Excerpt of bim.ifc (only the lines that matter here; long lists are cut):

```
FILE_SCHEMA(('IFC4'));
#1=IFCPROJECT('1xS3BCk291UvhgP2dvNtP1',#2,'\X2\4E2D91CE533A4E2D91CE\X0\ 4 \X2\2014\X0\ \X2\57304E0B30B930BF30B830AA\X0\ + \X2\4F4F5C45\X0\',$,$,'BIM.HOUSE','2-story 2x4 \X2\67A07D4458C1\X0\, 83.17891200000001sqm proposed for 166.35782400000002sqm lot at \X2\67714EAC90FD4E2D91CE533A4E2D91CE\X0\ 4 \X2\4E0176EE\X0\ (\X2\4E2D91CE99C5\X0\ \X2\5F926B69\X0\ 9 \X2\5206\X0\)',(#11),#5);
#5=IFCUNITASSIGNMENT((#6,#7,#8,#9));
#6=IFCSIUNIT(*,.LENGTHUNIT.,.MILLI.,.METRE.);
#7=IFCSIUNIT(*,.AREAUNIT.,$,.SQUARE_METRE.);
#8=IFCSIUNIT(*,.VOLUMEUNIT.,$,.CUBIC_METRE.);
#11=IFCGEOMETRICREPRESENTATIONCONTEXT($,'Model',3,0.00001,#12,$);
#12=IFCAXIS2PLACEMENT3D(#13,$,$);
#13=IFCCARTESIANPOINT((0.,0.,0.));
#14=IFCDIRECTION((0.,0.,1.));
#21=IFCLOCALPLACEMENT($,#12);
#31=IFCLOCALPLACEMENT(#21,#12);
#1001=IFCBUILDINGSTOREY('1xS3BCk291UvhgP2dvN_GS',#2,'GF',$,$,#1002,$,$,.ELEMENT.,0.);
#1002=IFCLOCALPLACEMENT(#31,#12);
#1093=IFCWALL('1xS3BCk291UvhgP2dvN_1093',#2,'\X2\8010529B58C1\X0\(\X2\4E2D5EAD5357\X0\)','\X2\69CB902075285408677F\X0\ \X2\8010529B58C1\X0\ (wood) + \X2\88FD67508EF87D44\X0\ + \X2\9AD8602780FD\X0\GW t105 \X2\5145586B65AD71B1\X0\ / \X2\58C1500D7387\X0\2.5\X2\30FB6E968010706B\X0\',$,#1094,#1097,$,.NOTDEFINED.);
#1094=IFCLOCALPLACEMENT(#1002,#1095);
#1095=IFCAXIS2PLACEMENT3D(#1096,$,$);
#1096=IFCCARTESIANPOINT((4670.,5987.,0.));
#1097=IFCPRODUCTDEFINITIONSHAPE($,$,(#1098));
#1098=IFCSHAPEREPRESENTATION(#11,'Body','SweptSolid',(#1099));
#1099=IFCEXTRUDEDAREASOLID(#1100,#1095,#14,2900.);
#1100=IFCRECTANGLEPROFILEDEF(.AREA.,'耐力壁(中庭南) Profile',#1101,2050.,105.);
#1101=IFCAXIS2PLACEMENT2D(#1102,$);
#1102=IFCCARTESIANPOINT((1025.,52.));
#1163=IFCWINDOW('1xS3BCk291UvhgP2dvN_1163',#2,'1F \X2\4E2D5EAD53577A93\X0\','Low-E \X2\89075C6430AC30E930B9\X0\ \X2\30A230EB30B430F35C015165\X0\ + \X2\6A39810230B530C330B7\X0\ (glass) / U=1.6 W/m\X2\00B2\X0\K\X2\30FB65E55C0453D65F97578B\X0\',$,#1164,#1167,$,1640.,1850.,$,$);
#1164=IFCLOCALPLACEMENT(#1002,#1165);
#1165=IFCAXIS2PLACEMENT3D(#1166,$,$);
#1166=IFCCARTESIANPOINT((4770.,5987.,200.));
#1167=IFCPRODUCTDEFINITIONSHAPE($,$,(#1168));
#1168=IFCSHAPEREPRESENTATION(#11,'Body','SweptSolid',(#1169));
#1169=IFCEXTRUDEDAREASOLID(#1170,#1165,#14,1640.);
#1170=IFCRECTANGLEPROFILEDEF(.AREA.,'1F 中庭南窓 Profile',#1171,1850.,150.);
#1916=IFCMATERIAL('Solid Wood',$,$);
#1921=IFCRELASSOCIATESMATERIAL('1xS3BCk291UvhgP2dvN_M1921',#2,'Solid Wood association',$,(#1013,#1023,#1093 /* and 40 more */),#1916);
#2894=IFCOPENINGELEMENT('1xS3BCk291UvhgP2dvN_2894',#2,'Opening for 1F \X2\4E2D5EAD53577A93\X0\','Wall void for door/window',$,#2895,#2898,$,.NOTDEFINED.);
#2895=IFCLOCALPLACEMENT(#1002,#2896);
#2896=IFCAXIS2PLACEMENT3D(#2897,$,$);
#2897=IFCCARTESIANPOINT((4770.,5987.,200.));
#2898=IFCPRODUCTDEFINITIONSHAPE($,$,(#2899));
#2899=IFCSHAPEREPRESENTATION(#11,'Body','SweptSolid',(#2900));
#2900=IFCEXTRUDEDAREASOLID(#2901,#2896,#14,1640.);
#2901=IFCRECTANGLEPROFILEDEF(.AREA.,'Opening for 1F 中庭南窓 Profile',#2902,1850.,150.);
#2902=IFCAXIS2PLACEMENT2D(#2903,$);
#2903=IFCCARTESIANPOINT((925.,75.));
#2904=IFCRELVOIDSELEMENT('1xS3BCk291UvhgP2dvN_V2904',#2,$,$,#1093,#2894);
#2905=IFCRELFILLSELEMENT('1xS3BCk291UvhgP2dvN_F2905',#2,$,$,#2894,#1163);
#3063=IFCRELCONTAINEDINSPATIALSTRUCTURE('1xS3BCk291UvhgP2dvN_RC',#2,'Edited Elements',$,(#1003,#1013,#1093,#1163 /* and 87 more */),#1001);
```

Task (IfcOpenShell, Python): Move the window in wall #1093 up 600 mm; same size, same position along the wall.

```python
import numpy as np
import ifcopenshell
import ifcopenshell.api.geometry
import ifcopenshell.util.placement
import ifcopenshell.util.unit

model = ifcopenshell.open("bim.ifc")
unit_scale = ifcopenshell.util.unit.calculate_unit_scale(model)

window = model.by_id(1163)
opening = window.FillsVoids[0].RelatingOpeningElement
dz = 0.6 / unit_scale

shift = np.array([0.0, 0.0, dz])
# The window is not placed relative to its opening, so move both.
for product in (opening, window):
    matrix = ifcopenshell.util.placement.get_local_placement(product.ObjectPlacement)
    matrix[:3, 3] += shift
    ifcopenshell.api.geometry.edit_object_placement(model, product=product, matrix=matrix, is_si=False)

print(f"moved by {dz * unit_scale:+.3f} m")

model.write("bim_v2.ifc")
```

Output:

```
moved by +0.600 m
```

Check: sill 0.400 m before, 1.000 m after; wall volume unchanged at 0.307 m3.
